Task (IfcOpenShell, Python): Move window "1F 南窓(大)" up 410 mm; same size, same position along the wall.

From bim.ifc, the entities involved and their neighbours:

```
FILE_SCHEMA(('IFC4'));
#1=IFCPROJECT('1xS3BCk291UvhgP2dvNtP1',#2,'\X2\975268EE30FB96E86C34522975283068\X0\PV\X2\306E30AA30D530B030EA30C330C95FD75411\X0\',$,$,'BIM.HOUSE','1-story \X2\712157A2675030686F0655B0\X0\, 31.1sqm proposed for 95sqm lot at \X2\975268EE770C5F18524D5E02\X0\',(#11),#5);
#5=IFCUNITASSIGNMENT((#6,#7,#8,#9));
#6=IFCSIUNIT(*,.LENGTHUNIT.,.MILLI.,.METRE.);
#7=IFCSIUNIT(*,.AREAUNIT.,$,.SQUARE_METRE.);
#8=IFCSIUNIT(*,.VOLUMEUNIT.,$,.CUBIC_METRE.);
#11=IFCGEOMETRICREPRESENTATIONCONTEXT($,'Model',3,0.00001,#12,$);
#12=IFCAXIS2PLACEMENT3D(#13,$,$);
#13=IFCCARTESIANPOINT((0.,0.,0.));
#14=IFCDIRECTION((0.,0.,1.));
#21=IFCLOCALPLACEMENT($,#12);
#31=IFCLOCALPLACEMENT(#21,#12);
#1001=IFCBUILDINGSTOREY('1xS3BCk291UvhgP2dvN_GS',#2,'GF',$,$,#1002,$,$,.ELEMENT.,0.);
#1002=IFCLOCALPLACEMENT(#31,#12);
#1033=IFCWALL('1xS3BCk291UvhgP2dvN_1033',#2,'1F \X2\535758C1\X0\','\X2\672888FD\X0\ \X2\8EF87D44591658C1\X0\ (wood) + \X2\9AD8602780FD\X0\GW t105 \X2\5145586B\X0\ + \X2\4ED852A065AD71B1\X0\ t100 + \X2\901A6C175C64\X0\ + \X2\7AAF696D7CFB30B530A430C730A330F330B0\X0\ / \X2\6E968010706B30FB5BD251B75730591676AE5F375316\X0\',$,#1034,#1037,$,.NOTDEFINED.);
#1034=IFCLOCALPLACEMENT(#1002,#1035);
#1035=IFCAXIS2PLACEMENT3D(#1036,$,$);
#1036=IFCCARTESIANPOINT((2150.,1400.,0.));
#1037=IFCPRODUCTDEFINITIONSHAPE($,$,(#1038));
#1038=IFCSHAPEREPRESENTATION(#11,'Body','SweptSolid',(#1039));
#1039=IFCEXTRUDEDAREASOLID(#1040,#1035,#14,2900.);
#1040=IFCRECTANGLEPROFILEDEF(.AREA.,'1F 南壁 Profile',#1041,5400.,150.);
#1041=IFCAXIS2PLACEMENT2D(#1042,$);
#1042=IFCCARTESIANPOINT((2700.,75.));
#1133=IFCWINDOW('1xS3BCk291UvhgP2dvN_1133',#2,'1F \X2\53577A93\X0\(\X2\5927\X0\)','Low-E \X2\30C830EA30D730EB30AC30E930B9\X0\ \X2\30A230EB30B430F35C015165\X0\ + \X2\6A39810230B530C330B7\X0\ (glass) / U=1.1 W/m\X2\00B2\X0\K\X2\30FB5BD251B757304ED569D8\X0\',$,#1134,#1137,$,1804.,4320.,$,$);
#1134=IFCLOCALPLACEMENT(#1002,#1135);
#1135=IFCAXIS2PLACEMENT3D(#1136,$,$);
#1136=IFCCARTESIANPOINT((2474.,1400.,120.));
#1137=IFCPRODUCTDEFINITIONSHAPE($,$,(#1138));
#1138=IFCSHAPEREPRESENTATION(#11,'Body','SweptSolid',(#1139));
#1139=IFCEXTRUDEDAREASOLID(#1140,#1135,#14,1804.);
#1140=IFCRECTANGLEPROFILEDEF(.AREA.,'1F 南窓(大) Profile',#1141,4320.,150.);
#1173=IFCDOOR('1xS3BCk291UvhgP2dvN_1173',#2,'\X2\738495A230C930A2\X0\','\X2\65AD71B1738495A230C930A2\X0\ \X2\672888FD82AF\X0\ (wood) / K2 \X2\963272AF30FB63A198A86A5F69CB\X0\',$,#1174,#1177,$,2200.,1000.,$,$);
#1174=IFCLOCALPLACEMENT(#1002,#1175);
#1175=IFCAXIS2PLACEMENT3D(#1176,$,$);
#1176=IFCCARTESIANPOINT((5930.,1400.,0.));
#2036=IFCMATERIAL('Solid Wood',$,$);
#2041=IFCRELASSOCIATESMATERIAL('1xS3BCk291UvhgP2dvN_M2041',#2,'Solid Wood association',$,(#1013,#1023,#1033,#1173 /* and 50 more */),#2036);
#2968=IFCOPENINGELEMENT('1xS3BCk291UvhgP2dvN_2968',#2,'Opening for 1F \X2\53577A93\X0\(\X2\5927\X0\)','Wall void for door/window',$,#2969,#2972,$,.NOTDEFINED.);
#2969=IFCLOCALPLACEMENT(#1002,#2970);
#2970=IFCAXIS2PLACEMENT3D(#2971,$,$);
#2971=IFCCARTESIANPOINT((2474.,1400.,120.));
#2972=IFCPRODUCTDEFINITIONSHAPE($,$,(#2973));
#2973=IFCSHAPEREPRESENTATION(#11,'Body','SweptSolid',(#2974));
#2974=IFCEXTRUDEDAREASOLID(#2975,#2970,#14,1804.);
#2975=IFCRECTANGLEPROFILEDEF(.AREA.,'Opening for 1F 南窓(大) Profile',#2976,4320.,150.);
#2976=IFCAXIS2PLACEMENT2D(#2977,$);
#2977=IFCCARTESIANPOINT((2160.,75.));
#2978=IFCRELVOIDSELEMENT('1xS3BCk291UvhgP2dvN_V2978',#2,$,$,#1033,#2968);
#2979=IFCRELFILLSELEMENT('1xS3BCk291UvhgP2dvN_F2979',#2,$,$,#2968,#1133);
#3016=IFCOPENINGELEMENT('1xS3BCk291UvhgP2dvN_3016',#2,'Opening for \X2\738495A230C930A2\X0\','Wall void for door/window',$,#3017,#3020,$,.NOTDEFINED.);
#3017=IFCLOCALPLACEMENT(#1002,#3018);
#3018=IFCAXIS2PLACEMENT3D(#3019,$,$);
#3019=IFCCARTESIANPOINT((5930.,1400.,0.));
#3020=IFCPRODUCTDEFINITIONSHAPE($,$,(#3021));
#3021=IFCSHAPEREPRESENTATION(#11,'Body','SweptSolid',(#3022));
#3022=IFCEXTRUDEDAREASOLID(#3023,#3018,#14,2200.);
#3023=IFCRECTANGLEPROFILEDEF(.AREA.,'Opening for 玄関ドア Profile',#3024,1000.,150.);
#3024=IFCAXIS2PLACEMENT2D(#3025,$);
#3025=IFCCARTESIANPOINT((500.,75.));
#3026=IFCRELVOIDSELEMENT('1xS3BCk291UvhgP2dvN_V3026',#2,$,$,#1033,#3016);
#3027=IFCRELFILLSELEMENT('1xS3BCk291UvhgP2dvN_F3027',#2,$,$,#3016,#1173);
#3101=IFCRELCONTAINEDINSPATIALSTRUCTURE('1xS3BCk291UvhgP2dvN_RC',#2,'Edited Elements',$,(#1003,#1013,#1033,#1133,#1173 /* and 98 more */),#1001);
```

```python
import numpy as np
import ifcopenshell
import ifcopenshell.api.geometry
import ifcopenshell.util.placement
import ifcopenshell.util.unit

model = ifcopenshell.open("bim.ifc")
unit_scale = ifcopenshell.util.unit.calculate_unit_scale(model)

window = model.by_id(1133)
opening = window.FillsVoids[0].RelatingOpeningElement
dz = 410.0

shift = np.array([0.0, 0.0, dz])
# The window is not placed relative to its opening, so move both.
for product in (opening, window):
    matrix = ifcopenshell.util.placement.get_local_placement(product.ObjectPlacement)
    matrix[:3, 3] += shift
    ifcopenshell.api.geometry.edit_object_placement(model, product=product, matrix=matrix, is_si=False)

print(f"moved by {dz * unit_scale:+.3f} m")

model.write("bim_edited.ifc")
```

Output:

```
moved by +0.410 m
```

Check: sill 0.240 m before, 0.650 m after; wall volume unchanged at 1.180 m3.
